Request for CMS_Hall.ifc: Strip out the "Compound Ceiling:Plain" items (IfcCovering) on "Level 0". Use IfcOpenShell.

First a look at what the model holds.

```python
import ifcopenshell
import ifcopenshell.util.element

model = ifcopenshell.open("CMS_Hall.ifc")
print(model.schema)
storey = next(s for s in model.by_type("IfcBuildingStorey") if s.Name == "Level 0")
coverings = [e for e in ifcopenshell.util.element.get_decomposition(storey) if e.is_a("IfcCovering")]
seen = {}
for e in coverings:
    element_type = ifcopenshell.util.element.get_type(e)
    name = element_type.Name if element_type not in (None, e) else None
    seen[name] = seen.get(name, 0) + 1
for name, count in sorted(seen.items(), key=str):
    print(count, "x", name)
```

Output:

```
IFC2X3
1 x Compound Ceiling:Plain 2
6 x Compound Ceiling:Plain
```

```python
import ifcopenshell
import ifcopenshell.api.root
import ifcopenshell.util.element

model = ifcopenshell.open("CMS_Hall.ifc")

storey = next(s for s in model.by_type("IfcBuildingStorey") if s.Name == "Level 0")
coverings = [e for e in ifcopenshell.util.element.get_decomposition(storey) if e.is_a("IfcCovering")]
targets = [e for e in coverings if (t := ifcopenshell.util.element.get_type(e)) not in (None, e) and t.Name == "Compound Ceiling:Plain"]

for e in targets:
    ifcopenshell.api.root.remove_product(model, product=e)
print(len(targets), "removed")

model.write("CMS_Hall_v2.ifc")
```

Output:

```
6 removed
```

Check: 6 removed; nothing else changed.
